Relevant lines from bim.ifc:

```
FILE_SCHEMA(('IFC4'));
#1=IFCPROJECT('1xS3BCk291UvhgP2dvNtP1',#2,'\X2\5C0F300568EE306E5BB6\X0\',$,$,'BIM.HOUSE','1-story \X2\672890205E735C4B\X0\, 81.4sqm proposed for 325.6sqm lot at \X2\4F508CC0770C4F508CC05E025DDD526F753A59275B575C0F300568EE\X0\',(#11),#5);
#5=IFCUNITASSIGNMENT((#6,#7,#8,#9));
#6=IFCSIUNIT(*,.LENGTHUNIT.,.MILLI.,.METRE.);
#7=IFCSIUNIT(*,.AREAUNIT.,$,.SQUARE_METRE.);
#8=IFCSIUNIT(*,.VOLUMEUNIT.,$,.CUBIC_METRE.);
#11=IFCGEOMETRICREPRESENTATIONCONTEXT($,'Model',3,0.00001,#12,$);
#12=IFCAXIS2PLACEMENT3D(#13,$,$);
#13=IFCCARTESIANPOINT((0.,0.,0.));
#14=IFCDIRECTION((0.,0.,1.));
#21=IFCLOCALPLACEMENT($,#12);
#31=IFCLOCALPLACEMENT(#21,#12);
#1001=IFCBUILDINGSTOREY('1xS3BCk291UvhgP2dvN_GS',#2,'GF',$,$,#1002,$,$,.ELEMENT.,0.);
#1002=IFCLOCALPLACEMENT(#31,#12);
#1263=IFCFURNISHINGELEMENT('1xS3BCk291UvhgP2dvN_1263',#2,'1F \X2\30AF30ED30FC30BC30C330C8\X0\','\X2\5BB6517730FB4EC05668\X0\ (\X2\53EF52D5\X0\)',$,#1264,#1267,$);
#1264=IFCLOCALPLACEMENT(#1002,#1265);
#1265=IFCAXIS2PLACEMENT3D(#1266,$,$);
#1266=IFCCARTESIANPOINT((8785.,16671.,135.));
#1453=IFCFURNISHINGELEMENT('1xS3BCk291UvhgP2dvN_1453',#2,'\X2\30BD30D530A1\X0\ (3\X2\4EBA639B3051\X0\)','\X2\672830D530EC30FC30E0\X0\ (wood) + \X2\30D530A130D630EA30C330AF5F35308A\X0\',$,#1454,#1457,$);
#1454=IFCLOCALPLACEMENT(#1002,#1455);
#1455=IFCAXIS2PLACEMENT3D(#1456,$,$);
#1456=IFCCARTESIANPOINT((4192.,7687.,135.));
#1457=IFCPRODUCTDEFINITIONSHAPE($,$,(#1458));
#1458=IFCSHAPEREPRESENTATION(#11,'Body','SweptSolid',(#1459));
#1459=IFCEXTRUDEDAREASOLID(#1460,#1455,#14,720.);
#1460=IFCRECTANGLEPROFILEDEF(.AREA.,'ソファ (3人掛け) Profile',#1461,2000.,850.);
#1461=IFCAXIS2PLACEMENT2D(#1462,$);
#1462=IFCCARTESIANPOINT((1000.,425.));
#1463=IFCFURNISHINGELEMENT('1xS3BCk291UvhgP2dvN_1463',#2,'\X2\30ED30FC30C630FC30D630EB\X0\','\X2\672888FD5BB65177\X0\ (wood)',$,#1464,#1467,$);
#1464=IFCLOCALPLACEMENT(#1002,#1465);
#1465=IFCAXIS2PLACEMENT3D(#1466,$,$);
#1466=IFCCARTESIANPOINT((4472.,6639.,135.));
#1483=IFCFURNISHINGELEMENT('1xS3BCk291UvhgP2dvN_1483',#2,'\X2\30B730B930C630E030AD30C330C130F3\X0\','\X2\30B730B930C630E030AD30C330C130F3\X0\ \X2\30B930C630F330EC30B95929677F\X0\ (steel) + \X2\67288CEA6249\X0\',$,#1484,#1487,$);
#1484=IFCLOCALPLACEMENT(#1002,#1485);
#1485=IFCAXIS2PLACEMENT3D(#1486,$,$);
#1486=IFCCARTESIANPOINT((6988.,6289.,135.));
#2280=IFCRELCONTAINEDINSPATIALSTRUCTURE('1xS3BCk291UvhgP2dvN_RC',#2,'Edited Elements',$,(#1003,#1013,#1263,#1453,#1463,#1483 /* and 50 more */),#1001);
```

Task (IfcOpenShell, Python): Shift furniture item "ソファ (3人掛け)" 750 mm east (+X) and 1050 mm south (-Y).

```python
import ifcopenshell
import ifcopenshell.api.geometry
import ifcopenshell.util.placement

model = ifcopenshell.open("bim.ifc")

item = model.by_guid("1xS3BCk291UvhgP2dvN_1453")
matrix = ifcopenshell.util.placement.get_local_placement(item.ObjectPlacement)
matrix[0, 3] += 750.0
matrix[1, 3] -= 1050.0
ifcopenshell.api.geometry.edit_object_placement(model, product=item, matrix=matrix, is_si=False)

print(ifcopenshell.util.placement.get_local_placement(item.ObjectPlacement).round(3) + 0.0)

model.write("bim_updated.ifc")
```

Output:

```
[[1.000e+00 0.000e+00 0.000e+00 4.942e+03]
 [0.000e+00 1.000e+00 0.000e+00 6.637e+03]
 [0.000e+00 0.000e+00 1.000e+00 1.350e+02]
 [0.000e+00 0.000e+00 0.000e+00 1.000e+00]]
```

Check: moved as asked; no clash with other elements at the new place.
